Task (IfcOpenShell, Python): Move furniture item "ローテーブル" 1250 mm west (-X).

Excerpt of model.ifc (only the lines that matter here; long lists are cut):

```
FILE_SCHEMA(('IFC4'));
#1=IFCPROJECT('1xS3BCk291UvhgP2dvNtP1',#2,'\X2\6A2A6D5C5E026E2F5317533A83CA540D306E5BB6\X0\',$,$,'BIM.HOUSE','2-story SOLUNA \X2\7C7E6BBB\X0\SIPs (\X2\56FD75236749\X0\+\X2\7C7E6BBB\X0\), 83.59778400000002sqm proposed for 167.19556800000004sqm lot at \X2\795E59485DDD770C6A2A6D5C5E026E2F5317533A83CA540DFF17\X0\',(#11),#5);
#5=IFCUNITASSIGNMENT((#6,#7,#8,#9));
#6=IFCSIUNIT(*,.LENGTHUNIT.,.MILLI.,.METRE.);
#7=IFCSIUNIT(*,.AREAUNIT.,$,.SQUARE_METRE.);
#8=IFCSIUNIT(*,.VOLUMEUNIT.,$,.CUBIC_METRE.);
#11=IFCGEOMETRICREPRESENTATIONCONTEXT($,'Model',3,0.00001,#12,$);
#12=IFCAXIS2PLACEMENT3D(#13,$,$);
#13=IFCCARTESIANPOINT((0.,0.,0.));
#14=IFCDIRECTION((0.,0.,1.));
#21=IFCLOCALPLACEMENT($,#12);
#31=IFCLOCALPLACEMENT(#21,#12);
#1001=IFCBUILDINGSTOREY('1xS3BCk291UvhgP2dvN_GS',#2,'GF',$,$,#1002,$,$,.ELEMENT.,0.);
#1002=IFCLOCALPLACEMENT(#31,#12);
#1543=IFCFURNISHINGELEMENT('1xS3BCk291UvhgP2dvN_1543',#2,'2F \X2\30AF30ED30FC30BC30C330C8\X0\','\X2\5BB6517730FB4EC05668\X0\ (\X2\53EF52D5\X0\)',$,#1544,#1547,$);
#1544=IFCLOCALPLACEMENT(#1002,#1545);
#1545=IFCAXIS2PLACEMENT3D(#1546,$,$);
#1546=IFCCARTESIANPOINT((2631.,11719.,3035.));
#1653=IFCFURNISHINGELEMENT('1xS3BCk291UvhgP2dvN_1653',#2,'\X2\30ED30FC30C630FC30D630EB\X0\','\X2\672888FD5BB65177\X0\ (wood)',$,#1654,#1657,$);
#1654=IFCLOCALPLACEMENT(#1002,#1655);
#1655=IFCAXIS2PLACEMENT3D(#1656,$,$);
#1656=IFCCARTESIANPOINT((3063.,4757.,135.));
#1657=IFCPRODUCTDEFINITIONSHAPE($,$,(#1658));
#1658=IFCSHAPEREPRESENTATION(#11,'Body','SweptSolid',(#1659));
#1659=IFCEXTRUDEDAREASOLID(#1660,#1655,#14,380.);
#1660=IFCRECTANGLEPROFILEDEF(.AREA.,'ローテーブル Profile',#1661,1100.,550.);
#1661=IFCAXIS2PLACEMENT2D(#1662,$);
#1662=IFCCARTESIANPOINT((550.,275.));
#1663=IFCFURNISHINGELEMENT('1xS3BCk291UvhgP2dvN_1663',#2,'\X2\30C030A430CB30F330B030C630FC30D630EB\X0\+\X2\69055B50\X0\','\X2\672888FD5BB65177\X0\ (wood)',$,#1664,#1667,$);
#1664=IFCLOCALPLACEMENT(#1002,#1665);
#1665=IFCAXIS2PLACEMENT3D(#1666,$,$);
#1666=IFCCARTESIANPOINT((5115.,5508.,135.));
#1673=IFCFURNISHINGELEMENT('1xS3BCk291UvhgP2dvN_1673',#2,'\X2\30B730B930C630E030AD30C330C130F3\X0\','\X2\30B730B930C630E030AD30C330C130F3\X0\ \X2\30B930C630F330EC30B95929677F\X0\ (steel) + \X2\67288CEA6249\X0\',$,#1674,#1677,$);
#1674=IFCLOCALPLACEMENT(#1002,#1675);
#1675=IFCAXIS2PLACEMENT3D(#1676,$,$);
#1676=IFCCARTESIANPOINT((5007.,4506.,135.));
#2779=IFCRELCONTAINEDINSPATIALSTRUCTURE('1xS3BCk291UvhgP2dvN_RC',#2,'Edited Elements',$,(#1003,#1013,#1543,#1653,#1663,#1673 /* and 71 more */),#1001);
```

```python
import ifcopenshell
import ifcopenshell.api.geometry
import ifcopenshell.util.placement
import ifcopenshell.util.unit

model = ifcopenshell.open("model.ifc")
unit_scale = ifcopenshell.util.unit.calculate_unit_scale(model)

item = model.by_id(1653)
matrix = ifcopenshell.util.placement.get_local_placement(item.ObjectPlacement)
matrix[0, 3] -= 1.25 / unit_scale
ifcopenshell.api.geometry.edit_object_placement(model, product=item, matrix=matrix, is_si=False)

print(ifcopenshell.util.placement.get_local_placement(item.ObjectPlacement).round(3) + 0.0)

model.write("model_v2.ifc")
```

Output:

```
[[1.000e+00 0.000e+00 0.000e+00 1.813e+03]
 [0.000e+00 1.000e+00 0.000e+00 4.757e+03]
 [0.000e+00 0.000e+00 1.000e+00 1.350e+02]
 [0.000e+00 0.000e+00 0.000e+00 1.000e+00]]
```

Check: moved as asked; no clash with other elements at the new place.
